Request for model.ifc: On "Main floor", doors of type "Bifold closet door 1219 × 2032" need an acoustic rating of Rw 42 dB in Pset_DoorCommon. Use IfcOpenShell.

First a look at what the model holds.

```python
import ifcopenshell
import ifcopenshell.util.element

model = ifcopenshell.open("model.ifc")
print(model.schema)
storey = next(s for s in model.by_type("IfcBuildingStorey") if s.Name == "Main floor")
doors = [e for e in ifcopenshell.util.element.get_decomposition(storey) if e.is_a("IfcDoor")]
seen = {}
for e in doors:
    element_type = ifcopenshell.util.element.get_type(e)
    key = (element_type.Name if element_type != e and element_type else None, ifcopenshell.util.element.get_pset(e, "Pset_DoorCommon", "AcousticRating"))
    seen[key] = seen.get(key, 0) + 1
for (name, value), count in sorted(seen.items(), key=str):
    print(count, "x", name, "|", value)
```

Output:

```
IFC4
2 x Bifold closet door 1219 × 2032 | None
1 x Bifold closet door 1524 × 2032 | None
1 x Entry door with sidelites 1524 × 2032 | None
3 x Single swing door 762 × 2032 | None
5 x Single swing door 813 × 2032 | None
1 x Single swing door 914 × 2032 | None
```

```python
import ifcopenshell
import ifcopenshell.api.pset
import ifcopenshell.util.element

model = ifcopenshell.open("model.ifc")

storey = next(s for s in model.by_type("IfcBuildingStorey") if s.Name == "Main floor")
doors = [e for e in ifcopenshell.util.element.get_decomposition(storey) if e.is_a("IfcDoor")]

count = 0
for e in doors:
    element_type = ifcopenshell.util.element.get_type(e)
    if element_type in (None, e) or element_type.Name != "Bifold closet door 1219 × 2032":
        continue
    # add_pset returns the element's existing set when there is one.
    pset = ifcopenshell.api.pset.add_pset(model, product=e, name="Pset_DoorCommon")
    ifcopenshell.api.pset.edit_pset(model, pset=pset, properties={"AcousticRating": "Rw 42 dB"})
    count += 1

print(count, "doors updated")

model.write("model_v2.ifc")
```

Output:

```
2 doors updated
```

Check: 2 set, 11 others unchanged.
